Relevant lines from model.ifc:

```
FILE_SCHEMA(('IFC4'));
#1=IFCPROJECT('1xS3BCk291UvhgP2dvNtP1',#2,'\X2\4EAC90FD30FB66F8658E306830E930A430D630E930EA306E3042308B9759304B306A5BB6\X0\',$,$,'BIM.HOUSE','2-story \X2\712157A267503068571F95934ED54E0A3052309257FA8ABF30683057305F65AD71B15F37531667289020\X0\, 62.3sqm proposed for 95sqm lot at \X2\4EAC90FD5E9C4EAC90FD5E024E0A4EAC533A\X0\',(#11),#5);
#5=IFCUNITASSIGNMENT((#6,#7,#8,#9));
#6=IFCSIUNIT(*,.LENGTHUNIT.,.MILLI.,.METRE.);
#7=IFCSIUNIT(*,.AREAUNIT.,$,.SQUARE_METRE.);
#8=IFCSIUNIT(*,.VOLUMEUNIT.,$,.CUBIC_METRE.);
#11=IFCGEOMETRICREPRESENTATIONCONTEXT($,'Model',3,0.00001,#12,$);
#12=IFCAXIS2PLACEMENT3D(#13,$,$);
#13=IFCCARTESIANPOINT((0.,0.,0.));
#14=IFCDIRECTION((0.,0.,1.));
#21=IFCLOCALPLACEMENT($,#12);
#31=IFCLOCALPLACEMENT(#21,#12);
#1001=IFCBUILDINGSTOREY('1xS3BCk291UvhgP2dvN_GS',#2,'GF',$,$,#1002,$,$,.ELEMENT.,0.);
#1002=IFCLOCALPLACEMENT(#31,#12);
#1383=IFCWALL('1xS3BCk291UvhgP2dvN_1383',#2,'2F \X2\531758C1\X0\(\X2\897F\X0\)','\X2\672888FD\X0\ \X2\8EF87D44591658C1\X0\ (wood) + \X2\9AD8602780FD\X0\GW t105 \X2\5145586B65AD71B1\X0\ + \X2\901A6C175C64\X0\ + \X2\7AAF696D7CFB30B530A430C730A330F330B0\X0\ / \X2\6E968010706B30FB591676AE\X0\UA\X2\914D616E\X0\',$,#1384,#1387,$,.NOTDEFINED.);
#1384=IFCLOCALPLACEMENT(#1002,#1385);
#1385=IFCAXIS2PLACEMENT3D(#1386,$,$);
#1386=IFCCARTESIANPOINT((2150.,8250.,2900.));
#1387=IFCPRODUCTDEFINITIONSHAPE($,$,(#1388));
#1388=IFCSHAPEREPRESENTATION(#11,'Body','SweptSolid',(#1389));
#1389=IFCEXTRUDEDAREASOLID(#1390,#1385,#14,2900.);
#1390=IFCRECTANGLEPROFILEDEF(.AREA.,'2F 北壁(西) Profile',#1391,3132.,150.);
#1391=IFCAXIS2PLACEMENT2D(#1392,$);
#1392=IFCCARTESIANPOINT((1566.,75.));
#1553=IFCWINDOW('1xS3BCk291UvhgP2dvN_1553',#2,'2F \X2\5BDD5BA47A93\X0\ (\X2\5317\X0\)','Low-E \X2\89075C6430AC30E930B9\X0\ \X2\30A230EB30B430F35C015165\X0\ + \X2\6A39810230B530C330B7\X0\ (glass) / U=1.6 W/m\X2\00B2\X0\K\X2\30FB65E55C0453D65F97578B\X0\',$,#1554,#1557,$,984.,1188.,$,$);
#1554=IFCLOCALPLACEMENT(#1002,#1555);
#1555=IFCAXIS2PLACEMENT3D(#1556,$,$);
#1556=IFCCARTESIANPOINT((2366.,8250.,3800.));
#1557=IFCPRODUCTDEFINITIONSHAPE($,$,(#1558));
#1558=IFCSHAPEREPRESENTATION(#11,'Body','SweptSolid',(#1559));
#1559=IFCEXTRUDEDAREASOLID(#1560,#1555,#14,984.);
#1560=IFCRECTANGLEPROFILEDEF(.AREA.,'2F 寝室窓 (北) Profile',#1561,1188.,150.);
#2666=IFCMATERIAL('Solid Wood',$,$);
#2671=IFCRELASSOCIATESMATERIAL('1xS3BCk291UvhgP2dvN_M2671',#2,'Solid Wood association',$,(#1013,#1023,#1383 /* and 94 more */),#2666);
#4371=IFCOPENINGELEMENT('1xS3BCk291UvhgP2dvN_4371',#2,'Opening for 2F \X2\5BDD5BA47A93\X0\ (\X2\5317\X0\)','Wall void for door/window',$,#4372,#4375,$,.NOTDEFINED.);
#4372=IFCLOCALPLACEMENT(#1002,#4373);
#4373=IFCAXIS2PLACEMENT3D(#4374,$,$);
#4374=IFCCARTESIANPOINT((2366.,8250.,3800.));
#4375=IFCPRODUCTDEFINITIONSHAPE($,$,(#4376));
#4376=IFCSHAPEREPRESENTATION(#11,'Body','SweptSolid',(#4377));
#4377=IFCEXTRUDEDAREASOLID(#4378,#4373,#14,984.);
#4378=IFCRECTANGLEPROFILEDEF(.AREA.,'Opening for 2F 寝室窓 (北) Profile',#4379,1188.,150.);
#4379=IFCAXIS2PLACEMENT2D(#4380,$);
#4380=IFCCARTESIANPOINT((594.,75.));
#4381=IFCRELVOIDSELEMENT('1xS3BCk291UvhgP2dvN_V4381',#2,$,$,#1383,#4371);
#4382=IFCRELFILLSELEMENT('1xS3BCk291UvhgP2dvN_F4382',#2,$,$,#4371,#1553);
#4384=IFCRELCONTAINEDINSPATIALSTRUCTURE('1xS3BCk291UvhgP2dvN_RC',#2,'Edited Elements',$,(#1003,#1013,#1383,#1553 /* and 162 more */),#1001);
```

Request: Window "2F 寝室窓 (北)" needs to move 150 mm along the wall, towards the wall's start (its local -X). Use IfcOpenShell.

```python
import ifcopenshell
import ifcopenshell.api.geometry
import ifcopenshell.util.placement
import ifcopenshell.util.unit

model = ifcopenshell.open("model.ifc")
unit_scale = ifcopenshell.util.unit.calculate_unit_scale(model)

window = model.by_guid("1xS3BCk291UvhgP2dvN_1553")
opening = window.FillsVoids[0].RelatingOpeningElement
wall = opening.VoidsElements[0].RelatingBuildingElement

wall_matrix = ifcopenshell.util.placement.get_local_placement(wall.ObjectPlacement)
shift = wall_matrix[:3, 0] * -0.15 / unit_scale
before = ifcopenshell.util.placement.get_local_placement(window.ObjectPlacement)[:3, 3].copy()

# The window is not placed relative to its opening, so move both.
for product in (opening, window):
    matrix = ifcopenshell.util.placement.get_local_placement(product.ObjectPlacement)
    matrix[:3, 3] += shift
    ifcopenshell.api.geometry.edit_object_placement(model, product=product, matrix=matrix, is_si=False)

after = ifcopenshell.util.placement.get_local_placement(window.ObjectPlacement)[:3, 3]
print("window moved by", (after - before).round(3) + 0.0)

model.write("model_v2.ifc")
```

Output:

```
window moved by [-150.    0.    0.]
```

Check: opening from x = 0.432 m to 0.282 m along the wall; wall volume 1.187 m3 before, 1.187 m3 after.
